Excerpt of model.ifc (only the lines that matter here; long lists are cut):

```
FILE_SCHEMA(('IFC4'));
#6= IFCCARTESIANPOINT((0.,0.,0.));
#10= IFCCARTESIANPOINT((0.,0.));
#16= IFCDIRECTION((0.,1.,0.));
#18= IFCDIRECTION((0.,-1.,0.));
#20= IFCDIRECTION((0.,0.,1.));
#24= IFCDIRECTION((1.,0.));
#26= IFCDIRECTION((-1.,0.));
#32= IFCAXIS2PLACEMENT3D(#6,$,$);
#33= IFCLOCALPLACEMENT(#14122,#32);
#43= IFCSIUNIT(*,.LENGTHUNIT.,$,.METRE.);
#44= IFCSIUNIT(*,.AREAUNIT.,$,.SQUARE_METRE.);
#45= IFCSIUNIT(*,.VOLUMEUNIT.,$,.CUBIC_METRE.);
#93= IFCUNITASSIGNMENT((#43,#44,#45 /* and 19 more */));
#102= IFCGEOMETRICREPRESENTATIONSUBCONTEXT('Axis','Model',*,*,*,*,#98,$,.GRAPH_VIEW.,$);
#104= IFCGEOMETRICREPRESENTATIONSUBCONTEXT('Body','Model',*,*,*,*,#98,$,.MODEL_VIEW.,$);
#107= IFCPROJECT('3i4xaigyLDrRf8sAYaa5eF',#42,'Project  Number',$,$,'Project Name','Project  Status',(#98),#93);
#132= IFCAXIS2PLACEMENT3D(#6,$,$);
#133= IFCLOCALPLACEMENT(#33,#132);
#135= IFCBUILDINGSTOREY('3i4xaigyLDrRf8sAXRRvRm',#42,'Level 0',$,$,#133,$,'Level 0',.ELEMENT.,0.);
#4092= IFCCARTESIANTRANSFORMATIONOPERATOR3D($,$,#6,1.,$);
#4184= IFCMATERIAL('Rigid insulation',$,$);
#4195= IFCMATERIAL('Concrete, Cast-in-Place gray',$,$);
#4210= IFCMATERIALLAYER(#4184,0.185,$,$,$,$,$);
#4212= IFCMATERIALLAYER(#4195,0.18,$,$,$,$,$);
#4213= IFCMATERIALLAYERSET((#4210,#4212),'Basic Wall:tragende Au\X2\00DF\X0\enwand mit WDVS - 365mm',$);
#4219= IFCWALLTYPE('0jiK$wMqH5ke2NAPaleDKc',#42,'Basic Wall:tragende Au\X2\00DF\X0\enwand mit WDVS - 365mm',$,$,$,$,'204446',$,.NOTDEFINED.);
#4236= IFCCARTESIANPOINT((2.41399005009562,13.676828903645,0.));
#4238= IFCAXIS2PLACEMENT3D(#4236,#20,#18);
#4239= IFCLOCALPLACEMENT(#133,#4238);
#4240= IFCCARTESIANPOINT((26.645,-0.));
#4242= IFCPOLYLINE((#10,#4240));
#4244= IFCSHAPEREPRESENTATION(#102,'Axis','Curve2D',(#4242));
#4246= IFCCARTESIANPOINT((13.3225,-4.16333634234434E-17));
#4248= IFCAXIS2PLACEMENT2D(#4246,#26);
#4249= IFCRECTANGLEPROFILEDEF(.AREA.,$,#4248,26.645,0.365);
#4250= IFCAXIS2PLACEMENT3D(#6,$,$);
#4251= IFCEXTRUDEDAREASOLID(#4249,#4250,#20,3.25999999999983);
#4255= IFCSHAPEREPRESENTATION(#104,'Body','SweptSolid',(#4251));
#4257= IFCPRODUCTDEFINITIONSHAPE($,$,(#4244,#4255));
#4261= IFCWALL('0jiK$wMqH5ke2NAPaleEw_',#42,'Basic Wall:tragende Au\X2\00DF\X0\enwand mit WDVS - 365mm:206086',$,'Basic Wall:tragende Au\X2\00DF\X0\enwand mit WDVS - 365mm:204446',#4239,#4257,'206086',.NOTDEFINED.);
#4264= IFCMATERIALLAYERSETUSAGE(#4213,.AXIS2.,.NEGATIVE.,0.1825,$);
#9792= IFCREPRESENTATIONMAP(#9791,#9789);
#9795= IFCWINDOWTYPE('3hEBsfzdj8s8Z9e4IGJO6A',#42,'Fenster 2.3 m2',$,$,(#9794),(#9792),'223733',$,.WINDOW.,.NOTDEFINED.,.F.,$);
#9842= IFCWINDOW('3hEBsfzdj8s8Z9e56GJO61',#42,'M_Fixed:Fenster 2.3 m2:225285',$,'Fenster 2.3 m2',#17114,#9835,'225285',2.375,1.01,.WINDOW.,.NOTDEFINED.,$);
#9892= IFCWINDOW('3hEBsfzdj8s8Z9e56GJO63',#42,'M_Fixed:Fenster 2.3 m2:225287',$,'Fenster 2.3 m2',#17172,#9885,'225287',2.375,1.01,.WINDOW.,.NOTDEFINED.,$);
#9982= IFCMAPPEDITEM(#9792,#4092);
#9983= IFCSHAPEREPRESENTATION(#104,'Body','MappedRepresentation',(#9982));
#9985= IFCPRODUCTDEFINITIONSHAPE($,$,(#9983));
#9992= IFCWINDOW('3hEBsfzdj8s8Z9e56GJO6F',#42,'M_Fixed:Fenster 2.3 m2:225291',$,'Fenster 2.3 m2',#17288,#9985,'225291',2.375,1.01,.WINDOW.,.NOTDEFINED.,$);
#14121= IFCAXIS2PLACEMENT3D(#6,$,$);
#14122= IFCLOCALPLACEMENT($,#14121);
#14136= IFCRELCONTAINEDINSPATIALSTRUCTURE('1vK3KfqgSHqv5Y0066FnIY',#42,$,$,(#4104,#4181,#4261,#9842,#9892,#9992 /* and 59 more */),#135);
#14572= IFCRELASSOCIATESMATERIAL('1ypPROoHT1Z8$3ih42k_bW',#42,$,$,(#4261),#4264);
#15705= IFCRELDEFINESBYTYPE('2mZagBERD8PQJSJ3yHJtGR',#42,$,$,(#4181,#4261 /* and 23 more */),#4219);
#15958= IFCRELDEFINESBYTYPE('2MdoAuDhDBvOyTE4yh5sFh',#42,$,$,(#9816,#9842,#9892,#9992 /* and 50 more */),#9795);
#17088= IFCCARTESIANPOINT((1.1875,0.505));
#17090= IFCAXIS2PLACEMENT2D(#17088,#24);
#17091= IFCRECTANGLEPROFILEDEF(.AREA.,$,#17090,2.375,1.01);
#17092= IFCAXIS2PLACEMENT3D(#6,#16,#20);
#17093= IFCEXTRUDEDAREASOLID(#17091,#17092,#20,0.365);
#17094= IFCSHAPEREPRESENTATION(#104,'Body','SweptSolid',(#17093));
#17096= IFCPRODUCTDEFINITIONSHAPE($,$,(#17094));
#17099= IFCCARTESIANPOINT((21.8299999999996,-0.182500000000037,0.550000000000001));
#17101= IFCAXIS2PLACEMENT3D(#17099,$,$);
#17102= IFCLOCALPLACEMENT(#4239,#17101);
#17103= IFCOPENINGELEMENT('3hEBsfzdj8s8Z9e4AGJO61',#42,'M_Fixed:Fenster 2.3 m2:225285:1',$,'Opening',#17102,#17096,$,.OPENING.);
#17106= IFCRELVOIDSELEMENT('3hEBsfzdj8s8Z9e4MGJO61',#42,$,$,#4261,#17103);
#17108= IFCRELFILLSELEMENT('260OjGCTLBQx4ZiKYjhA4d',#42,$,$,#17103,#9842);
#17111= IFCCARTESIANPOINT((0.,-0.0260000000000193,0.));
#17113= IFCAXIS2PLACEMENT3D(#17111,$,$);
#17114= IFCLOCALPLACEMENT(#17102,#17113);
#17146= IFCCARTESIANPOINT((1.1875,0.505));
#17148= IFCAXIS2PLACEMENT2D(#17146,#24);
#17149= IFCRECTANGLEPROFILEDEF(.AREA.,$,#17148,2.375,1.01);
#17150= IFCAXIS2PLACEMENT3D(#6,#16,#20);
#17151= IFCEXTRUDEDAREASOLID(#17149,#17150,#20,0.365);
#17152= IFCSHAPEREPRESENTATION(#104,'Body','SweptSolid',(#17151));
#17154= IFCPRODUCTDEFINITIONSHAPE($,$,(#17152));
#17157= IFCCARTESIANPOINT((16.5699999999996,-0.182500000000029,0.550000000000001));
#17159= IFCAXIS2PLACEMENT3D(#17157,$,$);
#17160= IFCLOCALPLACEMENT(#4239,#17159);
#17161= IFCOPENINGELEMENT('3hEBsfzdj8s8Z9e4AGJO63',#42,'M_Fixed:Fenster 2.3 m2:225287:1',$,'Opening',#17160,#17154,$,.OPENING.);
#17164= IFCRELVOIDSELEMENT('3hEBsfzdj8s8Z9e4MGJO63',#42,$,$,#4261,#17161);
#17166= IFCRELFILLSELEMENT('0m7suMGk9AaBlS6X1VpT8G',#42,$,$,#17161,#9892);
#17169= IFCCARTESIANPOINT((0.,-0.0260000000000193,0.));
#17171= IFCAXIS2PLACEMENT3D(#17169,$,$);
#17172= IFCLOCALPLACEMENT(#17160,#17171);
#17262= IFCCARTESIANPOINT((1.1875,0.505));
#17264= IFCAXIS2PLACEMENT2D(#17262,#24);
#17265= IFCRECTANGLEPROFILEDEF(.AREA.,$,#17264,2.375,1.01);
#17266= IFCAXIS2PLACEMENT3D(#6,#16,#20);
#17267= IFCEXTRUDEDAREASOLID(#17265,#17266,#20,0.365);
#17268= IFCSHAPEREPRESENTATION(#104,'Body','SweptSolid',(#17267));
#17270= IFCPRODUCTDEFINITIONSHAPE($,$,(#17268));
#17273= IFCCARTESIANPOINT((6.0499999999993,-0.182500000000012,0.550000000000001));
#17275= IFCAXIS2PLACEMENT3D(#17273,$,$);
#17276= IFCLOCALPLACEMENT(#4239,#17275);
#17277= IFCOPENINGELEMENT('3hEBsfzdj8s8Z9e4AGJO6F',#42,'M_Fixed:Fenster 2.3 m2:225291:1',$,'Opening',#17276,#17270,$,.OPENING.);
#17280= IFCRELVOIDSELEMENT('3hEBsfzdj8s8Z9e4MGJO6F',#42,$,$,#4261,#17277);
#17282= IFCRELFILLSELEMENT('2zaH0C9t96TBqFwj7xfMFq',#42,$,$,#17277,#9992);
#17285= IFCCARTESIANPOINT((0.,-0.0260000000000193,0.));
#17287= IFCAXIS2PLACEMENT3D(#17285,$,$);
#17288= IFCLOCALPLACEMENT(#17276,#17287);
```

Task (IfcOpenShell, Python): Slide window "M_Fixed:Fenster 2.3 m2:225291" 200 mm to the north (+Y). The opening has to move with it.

```python
import ifcopenshell
import ifcopenshell.api.geometry
import ifcopenshell.util.placement
import ifcopenshell.util.unit

model = ifcopenshell.open("model.ifc")
unit_scale = ifcopenshell.util.unit.calculate_unit_scale(model)

window = model.by_guid("3hEBsfzdj8s8Z9e56GJO6F")
opening = window.FillsVoids[0].RelatingOpeningElement
wall = opening.VoidsElements[0].RelatingBuildingElement

wall_matrix = ifcopenshell.util.placement.get_local_placement(wall.ObjectPlacement)
shift = wall_matrix[:3, 0] * -0.2 / unit_scale
before = ifcopenshell.util.placement.get_local_placement(window.ObjectPlacement)[:3, 3].copy()

# The window is placed relative to its opening, so it follows when the opening moves.
matrix = ifcopenshell.util.placement.get_local_placement(opening.ObjectPlacement)
matrix[:3, 3] += shift
ifcopenshell.api.geometry.edit_object_placement(
    model, product=opening, matrix=matrix, is_si=False, should_transform_children=True
)

after = ifcopenshell.util.placement.get_local_placement(window.ObjectPlacement)[:3, 3]
print("window moved by", (after - before).round(3) + 0.0)

model.write("model_v2.ifc")
```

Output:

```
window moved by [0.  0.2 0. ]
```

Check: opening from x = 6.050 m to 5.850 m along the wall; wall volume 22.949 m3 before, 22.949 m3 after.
